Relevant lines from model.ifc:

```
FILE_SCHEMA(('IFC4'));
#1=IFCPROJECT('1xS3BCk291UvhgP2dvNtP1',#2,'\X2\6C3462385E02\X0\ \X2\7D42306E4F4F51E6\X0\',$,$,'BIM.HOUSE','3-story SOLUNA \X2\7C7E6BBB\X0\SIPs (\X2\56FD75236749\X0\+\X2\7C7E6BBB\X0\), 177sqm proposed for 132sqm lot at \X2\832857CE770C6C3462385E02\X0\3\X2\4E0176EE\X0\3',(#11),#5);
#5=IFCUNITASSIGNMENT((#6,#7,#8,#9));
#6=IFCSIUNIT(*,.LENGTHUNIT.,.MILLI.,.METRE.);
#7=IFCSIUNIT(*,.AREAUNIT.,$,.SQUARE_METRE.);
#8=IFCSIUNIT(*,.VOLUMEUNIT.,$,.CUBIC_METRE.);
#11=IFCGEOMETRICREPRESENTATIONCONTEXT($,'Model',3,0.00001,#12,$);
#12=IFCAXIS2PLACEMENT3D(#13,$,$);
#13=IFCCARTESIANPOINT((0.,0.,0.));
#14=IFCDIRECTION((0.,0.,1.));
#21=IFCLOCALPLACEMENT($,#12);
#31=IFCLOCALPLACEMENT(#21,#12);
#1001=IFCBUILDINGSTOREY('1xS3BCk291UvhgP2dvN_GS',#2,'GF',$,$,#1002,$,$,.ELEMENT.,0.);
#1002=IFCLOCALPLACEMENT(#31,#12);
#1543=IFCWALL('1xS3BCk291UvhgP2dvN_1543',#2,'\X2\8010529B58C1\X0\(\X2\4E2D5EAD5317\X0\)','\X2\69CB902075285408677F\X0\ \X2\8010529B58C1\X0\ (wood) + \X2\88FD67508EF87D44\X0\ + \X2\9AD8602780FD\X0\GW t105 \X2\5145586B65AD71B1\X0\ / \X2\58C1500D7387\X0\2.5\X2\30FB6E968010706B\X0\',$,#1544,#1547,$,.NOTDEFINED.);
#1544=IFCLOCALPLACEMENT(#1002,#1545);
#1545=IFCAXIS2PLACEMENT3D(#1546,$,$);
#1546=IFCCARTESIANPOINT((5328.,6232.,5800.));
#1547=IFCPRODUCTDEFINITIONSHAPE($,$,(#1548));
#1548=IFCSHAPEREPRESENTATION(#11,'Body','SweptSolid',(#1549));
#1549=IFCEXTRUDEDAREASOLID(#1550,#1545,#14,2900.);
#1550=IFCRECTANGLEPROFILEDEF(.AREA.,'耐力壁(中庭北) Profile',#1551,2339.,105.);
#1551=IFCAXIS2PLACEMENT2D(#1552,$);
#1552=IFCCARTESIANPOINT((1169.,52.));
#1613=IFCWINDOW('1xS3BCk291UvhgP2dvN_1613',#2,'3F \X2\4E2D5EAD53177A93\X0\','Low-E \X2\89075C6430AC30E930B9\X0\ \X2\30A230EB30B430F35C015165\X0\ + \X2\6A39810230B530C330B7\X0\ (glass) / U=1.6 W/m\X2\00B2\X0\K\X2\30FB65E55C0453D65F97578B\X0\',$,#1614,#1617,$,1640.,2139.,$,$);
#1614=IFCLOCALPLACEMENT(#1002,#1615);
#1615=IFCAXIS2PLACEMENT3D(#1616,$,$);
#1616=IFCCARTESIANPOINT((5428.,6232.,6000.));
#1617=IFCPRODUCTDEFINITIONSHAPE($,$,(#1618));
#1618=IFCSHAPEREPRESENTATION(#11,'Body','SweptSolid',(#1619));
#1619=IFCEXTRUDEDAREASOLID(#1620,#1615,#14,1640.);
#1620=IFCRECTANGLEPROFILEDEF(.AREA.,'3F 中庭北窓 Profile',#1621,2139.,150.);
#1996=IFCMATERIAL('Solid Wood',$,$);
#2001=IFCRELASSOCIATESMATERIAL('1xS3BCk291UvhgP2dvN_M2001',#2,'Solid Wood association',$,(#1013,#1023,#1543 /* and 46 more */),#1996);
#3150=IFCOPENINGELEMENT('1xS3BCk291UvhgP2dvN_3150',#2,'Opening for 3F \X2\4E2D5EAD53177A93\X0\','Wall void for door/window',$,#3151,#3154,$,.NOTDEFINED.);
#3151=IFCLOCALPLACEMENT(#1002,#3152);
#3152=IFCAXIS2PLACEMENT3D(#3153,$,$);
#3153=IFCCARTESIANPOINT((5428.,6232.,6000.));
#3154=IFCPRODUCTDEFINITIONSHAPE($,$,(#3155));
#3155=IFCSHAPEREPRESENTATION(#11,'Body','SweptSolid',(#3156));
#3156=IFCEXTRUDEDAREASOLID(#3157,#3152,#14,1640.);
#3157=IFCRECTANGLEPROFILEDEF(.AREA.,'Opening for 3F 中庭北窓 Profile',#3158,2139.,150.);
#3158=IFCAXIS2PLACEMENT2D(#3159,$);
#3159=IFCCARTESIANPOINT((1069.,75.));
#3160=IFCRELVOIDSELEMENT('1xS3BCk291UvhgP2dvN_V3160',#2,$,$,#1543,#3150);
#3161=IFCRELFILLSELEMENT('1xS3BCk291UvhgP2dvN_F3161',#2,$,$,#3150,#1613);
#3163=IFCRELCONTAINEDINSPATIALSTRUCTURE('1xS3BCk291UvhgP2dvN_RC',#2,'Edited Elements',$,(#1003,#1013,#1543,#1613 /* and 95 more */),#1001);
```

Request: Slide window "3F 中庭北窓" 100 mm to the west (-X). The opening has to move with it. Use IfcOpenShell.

```python
import ifcopenshell
import ifcopenshell.api.geometry
import ifcopenshell.util.placement
import ifcopenshell.util.unit

model = ifcopenshell.open("model.ifc")
unit_scale = ifcopenshell.util.unit.calculate_unit_scale(model)

window = model.by_guid("1xS3BCk291UvhgP2dvN_1613")
opening = window.FillsVoids[0].RelatingOpeningElement
wall = opening.VoidsElements[0].RelatingBuildingElement

wall_matrix = ifcopenshell.util.placement.get_local_placement(wall.ObjectPlacement)
shift = wall_matrix[:3, 0] * -0.1 / unit_scale
before = ifcopenshell.util.placement.get_local_placement(window.ObjectPlacement)[:3, 3].copy()

# The window is not placed relative to its opening, so move both.
for product in (opening, window):
    matrix = ifcopenshell.util.placement.get_local_placement(product.ObjectPlacement)
    matrix[:3, 3] += shift
    ifcopenshell.api.geometry.edit_object_placement(model, product=product, matrix=matrix, is_si=False)

after = ifcopenshell.util.placement.get_local_placement(window.ObjectPlacement)[:3, 3]
print("window moved by", (after - before).round(3) + 0.0)

model.write("model_updated.ifc")
```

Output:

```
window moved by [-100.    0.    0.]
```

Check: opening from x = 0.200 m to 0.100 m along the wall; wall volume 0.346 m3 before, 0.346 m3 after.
